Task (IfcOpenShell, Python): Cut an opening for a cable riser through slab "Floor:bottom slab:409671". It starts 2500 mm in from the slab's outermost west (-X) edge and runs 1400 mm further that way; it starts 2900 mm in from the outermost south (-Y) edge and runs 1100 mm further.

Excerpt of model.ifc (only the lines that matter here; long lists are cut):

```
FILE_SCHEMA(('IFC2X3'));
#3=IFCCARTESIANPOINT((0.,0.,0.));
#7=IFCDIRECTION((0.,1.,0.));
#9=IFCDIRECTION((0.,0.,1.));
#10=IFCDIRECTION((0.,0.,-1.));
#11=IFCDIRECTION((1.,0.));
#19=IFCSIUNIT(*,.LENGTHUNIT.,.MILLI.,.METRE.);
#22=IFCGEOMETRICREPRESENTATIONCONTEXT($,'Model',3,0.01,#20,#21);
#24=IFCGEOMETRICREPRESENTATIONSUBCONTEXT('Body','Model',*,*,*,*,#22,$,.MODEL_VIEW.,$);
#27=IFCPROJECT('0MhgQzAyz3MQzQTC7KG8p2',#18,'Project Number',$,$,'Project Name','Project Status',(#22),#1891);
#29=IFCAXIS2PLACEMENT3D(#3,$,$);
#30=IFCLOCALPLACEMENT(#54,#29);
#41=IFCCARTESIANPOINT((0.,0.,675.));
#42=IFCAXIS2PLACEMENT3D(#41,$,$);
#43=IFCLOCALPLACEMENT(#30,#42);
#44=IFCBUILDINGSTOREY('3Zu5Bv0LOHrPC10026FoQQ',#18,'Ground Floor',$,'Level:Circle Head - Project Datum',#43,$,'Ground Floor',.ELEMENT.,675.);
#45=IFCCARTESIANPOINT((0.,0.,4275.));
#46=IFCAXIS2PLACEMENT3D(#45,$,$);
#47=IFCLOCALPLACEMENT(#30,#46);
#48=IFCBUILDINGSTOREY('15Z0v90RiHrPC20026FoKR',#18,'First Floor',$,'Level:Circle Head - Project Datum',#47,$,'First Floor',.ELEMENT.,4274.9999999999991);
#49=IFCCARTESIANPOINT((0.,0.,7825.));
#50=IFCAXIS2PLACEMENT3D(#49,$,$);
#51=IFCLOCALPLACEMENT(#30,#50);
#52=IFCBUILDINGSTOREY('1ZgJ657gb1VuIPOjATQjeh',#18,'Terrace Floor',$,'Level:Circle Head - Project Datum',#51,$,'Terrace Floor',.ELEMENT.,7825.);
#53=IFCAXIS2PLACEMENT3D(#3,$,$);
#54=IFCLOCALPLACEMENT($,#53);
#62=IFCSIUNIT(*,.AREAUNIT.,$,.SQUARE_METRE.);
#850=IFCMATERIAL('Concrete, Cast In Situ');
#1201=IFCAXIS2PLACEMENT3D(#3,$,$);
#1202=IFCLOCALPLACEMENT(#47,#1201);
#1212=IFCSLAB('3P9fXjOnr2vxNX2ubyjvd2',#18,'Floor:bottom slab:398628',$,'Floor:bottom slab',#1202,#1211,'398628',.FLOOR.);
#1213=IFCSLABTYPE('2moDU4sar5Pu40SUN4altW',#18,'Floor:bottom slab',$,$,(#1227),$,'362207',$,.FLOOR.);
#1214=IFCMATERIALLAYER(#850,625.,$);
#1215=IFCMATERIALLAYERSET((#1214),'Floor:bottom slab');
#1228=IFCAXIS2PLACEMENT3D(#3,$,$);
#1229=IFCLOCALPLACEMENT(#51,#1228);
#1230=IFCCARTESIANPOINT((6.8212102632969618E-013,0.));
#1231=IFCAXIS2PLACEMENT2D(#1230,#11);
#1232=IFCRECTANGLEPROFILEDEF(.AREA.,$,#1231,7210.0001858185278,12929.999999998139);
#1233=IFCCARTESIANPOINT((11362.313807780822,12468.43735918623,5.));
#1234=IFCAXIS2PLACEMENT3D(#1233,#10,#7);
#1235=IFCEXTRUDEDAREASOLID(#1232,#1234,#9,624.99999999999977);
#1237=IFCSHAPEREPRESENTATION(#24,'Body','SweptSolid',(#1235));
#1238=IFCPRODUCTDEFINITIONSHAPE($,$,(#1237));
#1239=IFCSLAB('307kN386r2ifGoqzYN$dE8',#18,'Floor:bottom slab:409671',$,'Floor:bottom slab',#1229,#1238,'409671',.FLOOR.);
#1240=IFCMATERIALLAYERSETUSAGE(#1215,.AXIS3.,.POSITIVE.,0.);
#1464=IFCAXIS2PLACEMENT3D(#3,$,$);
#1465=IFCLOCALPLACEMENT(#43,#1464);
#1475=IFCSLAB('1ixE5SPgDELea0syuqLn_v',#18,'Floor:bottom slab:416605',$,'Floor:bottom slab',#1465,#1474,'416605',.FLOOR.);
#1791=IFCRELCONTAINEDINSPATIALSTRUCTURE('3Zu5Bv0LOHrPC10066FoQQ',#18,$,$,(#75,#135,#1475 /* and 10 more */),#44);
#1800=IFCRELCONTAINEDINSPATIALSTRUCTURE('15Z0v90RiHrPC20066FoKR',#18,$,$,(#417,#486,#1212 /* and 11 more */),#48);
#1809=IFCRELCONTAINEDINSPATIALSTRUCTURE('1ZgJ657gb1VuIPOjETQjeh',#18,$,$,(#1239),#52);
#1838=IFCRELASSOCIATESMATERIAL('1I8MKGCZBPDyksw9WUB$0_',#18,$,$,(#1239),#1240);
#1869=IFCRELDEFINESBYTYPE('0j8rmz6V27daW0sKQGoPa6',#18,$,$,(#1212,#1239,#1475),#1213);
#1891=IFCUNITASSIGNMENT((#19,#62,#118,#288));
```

```python
import numpy as np
import ifcopenshell
import ifcopenshell.api.feature
import ifcopenshell.api.geometry
import ifcopenshell.api.root
import ifcopenshell.geom
import ifcopenshell.util.placement
import ifcopenshell.util.representation
import ifcopenshell.util.shape
import ifcopenshell.util.unit

model = ifcopenshell.open("model.ifc")
unit_scale = ifcopenshell.util.unit.calculate_unit_scale(model)
settings = ifcopenshell.geom.settings()


def volume(element):
    """Net volume in cubic metres, openings subtracted."""
    shape = ifcopenshell.geom.create_shape(settings, element)
    return ifcopenshell.util.shape.get_volume(shape.geometry)


slab = model.by_guid("307kN386r2ifGoqzYN$dE8")
before = volume(slab)

# Extent in the slab's own axes, in metres. The edges named are its -X and -Y sides.
slab_shape = ifcopenshell.geom.create_shape(settings, slab)
vertices = ifcopenshell.util.shape.get_vertices(slab_shape.geometry)
x_min, y_min, bottom = vertices.min(axis=0)
top = vertices[:, 2].max()

opening = ifcopenshell.api.root.create_entity(model, ifc_class="IfcOpeningElement", name="Cable riser opening")
context = ifcopenshell.util.representation.get_context(model, "Model", "Body", "MODEL_VIEW")
width, depth = 1.4, 1.1
outline = [(0.0, 0.0), (width, 0.0), (width, depth), (0.0, depth), (0.0, 0.0)]
# Overshoot both faces by 50 mm so the cut is clean.
shape = ifcopenshell.api.geometry.add_slab_representation(
    model, context=context, depth=top - bottom + 0.1, polyline=outline
)
ifcopenshell.api.geometry.assign_representation(model, product=opening, representation=shape)

matrix = ifcopenshell.util.placement.get_local_placement(slab.ObjectPlacement)
matrix[:, 3] = matrix @ np.append(np.array([x_min + 2.5, y_min + 2.9, bottom - 0.05]) / unit_scale, 1.0)
ifcopenshell.api.geometry.edit_object_placement(model, product=opening, matrix=matrix, is_si=False)
ifcopenshell.api.feature.add_feature(model, feature=opening, element=slab)

after = volume(slab)

print(f"slab volume {before:.3f} -> {after:.3f} m3")

model.write("model_updated.ifc")
```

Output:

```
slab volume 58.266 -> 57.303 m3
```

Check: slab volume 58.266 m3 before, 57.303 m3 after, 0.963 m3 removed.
